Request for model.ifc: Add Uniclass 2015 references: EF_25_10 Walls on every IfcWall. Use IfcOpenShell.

First a look at what the model holds.

```python
import ifcopenshell

model = ifcopenshell.open("model.ifc")
print(model.schema)
print("classifications:", [c.Name for c in model.by_type("IfcClassification")])
for ifc_class in ("IfcDoor", "IfcRoof", "IfcStair", "IfcWall", "IfcWindow"):
    print(ifc_class, len(model.by_type(ifc_class)))
```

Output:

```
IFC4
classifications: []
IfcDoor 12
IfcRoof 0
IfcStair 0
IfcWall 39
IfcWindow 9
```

```python
import ifcopenshell
import ifcopenshell.api.classification

model = ifcopenshell.open("model.ifc")

system = ifcopenshell.api.classification.add_classification(model, classification="Uniclass 2015")

codes = {
    "IfcWall": ("EF_25_10", "Walls"),
}
for ifc_class, (code, name) in codes.items():
    products = model.by_type(ifc_class)
    ifcopenshell.api.classification.add_reference(
        model, products=products, classification=system, identification=code, name=name
    )
    print(code, len(products))

model.write("model_v2.ifc")
```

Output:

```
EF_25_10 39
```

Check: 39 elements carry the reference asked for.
